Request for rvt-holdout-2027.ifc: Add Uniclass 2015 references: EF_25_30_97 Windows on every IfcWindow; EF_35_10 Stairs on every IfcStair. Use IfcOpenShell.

First a look at what the model holds.

```python
import ifcopenshell

model = ifcopenshell.open("rvt-holdout-2027.ifc")
print(model.schema)
print("classifications:", [c.Name for c in model.by_type("IfcClassification")])
for ifc_class in ("IfcDoor", "IfcRoof", "IfcStair", "IfcWall", "IfcWindow"):
    print(ifc_class, len(model.by_type(ifc_class)))
```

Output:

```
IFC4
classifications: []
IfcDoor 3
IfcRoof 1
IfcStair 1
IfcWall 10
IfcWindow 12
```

```python
import ifcopenshell
import ifcopenshell.api.classification

model = ifcopenshell.open("rvt-holdout-2027.ifc")

system = ifcopenshell.api.classification.add_classification(model, classification="Uniclass 2015")

codes = {
    "IfcWindow": ("EF_25_30_97", "Windows"),
    "IfcStair": ("EF_35_10", "Stairs"),
}
for ifc_class, (code, name) in codes.items():
    products = model.by_type(ifc_class)
    ifcopenshell.api.classification.add_reference(
        model, products=products, classification=system, identification=code, name=name
    )
    print(code, len(products))

model.write("rvt-holdout-2027-out.ifc")
```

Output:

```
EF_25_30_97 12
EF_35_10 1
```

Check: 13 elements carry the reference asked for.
